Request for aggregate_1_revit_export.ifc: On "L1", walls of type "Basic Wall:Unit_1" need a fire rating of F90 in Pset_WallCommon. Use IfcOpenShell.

First a look at what the model holds.

```python
import ifcopenshell
import ifcopenshell.util.element

model = ifcopenshell.open("aggregate_1_revit_export.ifc")
print(model.schema)
storey = next(s for s in model.by_type("IfcBuildingStorey") if s.Name == "L1")
walls = [e for e in ifcopenshell.util.element.get_decomposition(storey) if e.is_a("IfcWall")]
seen = {}
for e in walls:
    element_type = ifcopenshell.util.element.get_type(e)
    key = (element_type.Name if element_type != e and element_type else None, ifcopenshell.util.element.get_pset(e, "Pset_WallCommon", "FireRating"))
    seen[key] = seen.get(key, 0) + 1
for (name, value), count in sorted(seen.items(), key=str):
    print(count, "x", name, "|", value)
```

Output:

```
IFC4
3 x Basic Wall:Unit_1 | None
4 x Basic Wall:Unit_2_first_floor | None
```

```python
import ifcopenshell
import ifcopenshell.api.pset
import ifcopenshell.util.element

model = ifcopenshell.open("aggregate_1_revit_export.ifc")

storey = next(s for s in model.by_type("IfcBuildingStorey") if s.Name == "L1")
walls = [e for e in ifcopenshell.util.element.get_decomposition(storey) if e.is_a("IfcWall")]

count = 0
for e in walls:
    element_type = ifcopenshell.util.element.get_type(e)
    if element_type in (None, e) or element_type.Name != "Basic Wall:Unit_1":
        continue
    # add_pset returns the element's existing set when there is one.
    pset = ifcopenshell.api.pset.add_pset(model, product=e, name="Pset_WallCommon")
    ifcopenshell.api.pset.edit_pset(model, pset=pset, properties={"FireRating": "F90"})
    count += 1

print(count, "walls updated")

model.write("aggregate_1_revit_export_v2.ifc")
```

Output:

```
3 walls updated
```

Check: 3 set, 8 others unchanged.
